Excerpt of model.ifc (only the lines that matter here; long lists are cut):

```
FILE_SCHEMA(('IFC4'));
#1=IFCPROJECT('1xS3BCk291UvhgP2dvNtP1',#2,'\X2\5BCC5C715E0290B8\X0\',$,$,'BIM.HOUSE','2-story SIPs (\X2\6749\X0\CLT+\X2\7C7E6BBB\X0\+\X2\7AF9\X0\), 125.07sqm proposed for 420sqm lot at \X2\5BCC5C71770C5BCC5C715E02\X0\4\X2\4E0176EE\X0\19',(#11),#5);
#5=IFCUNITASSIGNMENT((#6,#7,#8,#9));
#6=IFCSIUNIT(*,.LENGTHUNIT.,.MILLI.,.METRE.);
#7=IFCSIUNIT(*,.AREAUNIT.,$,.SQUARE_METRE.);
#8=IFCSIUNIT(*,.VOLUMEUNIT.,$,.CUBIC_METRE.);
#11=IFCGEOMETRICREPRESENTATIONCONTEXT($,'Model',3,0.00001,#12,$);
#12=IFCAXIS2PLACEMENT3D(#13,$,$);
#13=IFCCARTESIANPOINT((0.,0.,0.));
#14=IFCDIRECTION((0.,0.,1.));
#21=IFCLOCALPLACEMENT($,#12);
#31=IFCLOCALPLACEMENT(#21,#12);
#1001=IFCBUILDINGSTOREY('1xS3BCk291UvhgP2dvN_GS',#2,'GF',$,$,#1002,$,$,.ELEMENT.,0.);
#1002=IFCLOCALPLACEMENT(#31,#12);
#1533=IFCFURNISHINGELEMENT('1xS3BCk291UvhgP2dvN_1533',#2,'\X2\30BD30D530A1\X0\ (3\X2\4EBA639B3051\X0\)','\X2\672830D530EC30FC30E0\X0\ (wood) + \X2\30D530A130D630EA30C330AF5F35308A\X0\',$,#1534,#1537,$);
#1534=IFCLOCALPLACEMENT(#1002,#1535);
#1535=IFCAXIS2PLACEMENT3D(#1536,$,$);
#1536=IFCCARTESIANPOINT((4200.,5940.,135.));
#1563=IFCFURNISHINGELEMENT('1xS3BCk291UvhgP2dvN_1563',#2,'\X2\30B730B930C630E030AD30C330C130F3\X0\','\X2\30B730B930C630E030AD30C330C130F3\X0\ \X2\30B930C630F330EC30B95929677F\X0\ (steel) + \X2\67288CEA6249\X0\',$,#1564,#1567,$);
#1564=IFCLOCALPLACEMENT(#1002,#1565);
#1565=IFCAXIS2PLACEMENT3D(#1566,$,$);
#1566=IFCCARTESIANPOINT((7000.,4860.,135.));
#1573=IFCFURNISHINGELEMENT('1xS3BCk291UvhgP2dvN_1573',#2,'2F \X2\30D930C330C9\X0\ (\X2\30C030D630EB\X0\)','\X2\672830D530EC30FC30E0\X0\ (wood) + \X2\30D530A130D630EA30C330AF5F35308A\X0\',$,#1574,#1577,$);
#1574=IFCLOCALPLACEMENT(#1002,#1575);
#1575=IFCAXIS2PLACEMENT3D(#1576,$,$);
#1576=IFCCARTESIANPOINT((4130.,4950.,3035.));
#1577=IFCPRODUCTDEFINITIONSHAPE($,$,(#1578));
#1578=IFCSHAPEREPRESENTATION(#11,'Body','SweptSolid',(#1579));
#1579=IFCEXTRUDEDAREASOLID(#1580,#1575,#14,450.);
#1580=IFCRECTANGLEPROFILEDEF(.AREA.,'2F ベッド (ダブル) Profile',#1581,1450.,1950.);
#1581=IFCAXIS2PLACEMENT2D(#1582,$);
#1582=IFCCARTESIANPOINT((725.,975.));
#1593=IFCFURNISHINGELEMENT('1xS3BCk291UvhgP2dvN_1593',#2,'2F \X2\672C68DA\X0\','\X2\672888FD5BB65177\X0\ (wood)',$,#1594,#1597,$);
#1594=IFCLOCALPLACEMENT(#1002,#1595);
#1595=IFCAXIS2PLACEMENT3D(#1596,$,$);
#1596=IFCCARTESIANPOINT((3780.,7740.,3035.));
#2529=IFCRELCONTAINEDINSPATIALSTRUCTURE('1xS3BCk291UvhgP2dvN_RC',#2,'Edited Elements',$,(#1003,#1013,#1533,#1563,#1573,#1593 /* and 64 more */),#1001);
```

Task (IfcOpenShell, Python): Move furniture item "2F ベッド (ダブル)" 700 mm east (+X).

```python
import ifcopenshell
import ifcopenshell.api.geometry
import ifcopenshell.util.placement
import ifcopenshell.util.unit

model = ifcopenshell.open("model.ifc")
unit_scale = ifcopenshell.util.unit.calculate_unit_scale(model)

item = model.by_guid("1xS3BCk291UvhgP2dvN_1573")
matrix = ifcopenshell.util.placement.get_local_placement(item.ObjectPlacement)
matrix[0, 3] += 0.7 / unit_scale
ifcopenshell.api.geometry.edit_object_placement(model, product=item, matrix=matrix, is_si=False)

print(ifcopenshell.util.placement.get_local_placement(item.ObjectPlacement).round(3) + 0.0)

model.write("model-out.ifc")
```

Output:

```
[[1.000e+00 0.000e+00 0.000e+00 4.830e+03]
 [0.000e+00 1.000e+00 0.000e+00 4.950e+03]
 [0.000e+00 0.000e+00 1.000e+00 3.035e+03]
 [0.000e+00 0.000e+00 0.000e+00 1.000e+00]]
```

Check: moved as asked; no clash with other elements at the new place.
